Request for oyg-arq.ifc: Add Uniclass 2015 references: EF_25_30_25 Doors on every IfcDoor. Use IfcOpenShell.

First a look at what the model holds.

```python
import ifcopenshell

model = ifcopenshell.open("oyg-arq.ifc")
print(model.schema)
print("classifications:", [c.Name for c in model.by_type("IfcClassification")])
for ifc_class in ("IfcDoor", "IfcRoof", "IfcStair", "IfcWall", "IfcWindow"):
    print(ifc_class, len(model.by_type(ifc_class)))
```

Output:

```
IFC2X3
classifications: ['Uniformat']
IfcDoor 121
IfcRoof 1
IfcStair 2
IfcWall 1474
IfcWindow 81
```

```python
import ifcopenshell
import ifcopenshell.api.classification

model = ifcopenshell.open("oyg-arq.ifc")

# IFC2X3 requires Source and Edition and has no link from the project to the system.
system = model.create_entity("IfcClassification", Source="NBS", Edition="2015", Name="Uniclass 2015")

codes = {
    "IfcDoor": ("EF_25_30_25", "Doors"),
}
for ifc_class, (code, name) in codes.items():
    products = model.by_type(ifc_class)
    ifcopenshell.api.classification.add_reference(
        model, products=products, classification=system, identification=code, name=name
    )
    print(code, len(products))

model.write("oyg-arq_edited.ifc")
```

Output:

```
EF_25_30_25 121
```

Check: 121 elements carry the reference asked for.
